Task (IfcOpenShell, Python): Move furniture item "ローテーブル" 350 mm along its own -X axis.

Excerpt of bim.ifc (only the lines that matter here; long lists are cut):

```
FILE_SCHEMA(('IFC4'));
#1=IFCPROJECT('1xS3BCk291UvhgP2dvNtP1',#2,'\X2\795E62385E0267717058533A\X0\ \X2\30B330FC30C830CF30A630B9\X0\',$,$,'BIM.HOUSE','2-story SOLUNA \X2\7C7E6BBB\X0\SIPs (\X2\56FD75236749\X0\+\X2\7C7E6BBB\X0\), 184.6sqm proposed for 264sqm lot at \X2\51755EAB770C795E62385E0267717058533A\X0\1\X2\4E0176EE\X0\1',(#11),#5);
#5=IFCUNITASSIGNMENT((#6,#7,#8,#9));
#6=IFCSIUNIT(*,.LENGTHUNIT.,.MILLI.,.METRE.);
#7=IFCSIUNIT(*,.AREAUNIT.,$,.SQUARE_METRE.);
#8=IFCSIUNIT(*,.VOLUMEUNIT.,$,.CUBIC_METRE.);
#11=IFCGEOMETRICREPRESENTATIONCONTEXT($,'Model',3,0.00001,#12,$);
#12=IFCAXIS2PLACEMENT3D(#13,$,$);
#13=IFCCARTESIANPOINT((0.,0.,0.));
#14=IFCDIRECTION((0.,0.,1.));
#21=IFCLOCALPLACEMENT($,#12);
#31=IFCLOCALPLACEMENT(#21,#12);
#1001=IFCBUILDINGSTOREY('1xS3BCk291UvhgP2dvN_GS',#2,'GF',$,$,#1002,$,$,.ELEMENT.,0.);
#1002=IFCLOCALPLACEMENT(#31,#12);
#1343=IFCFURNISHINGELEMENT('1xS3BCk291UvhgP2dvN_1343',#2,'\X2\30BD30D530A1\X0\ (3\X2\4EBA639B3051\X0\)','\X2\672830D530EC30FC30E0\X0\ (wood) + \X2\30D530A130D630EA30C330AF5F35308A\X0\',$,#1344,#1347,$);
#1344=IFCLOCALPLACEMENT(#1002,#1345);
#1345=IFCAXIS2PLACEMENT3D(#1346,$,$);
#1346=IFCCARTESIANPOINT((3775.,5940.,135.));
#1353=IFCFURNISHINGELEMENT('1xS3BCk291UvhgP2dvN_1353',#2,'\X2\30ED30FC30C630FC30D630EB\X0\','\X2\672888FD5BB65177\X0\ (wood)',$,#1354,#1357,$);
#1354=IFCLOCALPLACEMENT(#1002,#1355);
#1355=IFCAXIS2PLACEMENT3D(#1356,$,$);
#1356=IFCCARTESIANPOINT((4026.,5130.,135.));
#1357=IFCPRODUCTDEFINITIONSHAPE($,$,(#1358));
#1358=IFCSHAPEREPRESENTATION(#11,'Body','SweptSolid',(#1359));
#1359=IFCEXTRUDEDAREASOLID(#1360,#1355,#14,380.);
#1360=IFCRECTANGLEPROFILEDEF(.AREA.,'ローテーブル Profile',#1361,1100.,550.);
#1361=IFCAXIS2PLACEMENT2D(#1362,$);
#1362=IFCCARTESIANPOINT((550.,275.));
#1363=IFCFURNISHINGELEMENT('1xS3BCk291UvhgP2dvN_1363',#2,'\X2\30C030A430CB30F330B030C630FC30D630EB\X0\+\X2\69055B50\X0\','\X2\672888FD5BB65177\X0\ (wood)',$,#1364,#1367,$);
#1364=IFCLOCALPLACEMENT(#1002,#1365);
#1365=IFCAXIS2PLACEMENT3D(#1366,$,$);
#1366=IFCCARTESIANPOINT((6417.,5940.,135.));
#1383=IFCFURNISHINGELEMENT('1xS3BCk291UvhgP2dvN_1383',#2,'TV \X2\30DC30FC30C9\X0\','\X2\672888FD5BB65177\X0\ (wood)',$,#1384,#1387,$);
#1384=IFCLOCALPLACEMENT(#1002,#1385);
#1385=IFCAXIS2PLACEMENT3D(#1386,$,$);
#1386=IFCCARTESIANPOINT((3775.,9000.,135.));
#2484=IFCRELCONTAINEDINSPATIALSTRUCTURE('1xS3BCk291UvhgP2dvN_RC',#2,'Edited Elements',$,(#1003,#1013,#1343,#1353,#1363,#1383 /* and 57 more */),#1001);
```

```python
import ifcopenshell
import ifcopenshell.api.geometry
import ifcopenshell.util.placement

model = ifcopenshell.open("bim.ifc")

item = model.by_guid("1xS3BCk291UvhgP2dvN_1353")
matrix = ifcopenshell.util.placement.get_local_placement(item.ObjectPlacement)
matrix[:3, 3] -= matrix[:3, 0] * 350.0
ifcopenshell.api.geometry.edit_object_placement(model, product=item, matrix=matrix, is_si=False)

print(ifcopenshell.util.placement.get_local_placement(item.ObjectPlacement).round(3) + 0.0)

model.write("bim_edited.ifc")
```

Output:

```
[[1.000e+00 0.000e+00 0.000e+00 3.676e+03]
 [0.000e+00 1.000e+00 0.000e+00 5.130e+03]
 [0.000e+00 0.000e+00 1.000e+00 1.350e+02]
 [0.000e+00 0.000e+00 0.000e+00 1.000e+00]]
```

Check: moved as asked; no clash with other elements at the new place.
